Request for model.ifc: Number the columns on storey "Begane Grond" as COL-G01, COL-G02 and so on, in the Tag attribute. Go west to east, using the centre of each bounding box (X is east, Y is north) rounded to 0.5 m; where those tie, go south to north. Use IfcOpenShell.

First a look at what the model holds.

```python
import ifcopenshell
import ifcopenshell.util.element
import ifcopenshell.util.placement

model = ifcopenshell.open("model.ifc")
print(model.schema)
storey = next(s for s in model.by_type("IfcBuildingStorey") if s.Name == "Begane Grond")
columns = [e for e in ifcopenshell.util.element.get_decomposition(storey) if e.is_a("IfcColumn")]
for e in sorted(columns, key=lambda e: e.id()):
    origin = ifcopenshell.util.placement.get_local_placement(e.ObjectPlacement)[:3, 3]
    print(e.id(), e.Tag, e.Name, origin.round(2) + 0.0, sep=" | ")
```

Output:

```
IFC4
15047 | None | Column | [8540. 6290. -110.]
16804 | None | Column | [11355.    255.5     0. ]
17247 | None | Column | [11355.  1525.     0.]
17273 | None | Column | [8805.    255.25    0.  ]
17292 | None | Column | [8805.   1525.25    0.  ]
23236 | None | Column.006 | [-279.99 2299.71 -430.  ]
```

```python
import ifcopenshell
import ifcopenshell.geom
import ifcopenshell.util.element
import ifcopenshell.util.shape

model = ifcopenshell.open("model.ifc")
settings = ifcopenshell.geom.settings()
settings.set("use-world-coords", True)


def centre(element):
    shape = ifcopenshell.geom.create_shape(settings, element)
    return ifcopenshell.util.shape.get_bbox_centroid(shape.geometry)


storey = next(s for s in model.by_type("IfcBuildingStorey") if s.Name == "Begane Grond")
columns = [e for e in ifcopenshell.util.element.get_decomposition(storey) if e.is_a("IfcColumn")]

# Insertion points can sit at a corner or the storey origin, so sort by the geometry (in metres).
centres = {e: centre(e) for e in columns}
columns.sort(key=lambda e: (round(centres[e][0] / 0.5), centres[e][1]))

for i, e in enumerate(columns, start=1):
    number = f"COL-G{i:02d}"
    e.Tag = number
    print(e.id(), number)

model.write("model_rev.ifc")
```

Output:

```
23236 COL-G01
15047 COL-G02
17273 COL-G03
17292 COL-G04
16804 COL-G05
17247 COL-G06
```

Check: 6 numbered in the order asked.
